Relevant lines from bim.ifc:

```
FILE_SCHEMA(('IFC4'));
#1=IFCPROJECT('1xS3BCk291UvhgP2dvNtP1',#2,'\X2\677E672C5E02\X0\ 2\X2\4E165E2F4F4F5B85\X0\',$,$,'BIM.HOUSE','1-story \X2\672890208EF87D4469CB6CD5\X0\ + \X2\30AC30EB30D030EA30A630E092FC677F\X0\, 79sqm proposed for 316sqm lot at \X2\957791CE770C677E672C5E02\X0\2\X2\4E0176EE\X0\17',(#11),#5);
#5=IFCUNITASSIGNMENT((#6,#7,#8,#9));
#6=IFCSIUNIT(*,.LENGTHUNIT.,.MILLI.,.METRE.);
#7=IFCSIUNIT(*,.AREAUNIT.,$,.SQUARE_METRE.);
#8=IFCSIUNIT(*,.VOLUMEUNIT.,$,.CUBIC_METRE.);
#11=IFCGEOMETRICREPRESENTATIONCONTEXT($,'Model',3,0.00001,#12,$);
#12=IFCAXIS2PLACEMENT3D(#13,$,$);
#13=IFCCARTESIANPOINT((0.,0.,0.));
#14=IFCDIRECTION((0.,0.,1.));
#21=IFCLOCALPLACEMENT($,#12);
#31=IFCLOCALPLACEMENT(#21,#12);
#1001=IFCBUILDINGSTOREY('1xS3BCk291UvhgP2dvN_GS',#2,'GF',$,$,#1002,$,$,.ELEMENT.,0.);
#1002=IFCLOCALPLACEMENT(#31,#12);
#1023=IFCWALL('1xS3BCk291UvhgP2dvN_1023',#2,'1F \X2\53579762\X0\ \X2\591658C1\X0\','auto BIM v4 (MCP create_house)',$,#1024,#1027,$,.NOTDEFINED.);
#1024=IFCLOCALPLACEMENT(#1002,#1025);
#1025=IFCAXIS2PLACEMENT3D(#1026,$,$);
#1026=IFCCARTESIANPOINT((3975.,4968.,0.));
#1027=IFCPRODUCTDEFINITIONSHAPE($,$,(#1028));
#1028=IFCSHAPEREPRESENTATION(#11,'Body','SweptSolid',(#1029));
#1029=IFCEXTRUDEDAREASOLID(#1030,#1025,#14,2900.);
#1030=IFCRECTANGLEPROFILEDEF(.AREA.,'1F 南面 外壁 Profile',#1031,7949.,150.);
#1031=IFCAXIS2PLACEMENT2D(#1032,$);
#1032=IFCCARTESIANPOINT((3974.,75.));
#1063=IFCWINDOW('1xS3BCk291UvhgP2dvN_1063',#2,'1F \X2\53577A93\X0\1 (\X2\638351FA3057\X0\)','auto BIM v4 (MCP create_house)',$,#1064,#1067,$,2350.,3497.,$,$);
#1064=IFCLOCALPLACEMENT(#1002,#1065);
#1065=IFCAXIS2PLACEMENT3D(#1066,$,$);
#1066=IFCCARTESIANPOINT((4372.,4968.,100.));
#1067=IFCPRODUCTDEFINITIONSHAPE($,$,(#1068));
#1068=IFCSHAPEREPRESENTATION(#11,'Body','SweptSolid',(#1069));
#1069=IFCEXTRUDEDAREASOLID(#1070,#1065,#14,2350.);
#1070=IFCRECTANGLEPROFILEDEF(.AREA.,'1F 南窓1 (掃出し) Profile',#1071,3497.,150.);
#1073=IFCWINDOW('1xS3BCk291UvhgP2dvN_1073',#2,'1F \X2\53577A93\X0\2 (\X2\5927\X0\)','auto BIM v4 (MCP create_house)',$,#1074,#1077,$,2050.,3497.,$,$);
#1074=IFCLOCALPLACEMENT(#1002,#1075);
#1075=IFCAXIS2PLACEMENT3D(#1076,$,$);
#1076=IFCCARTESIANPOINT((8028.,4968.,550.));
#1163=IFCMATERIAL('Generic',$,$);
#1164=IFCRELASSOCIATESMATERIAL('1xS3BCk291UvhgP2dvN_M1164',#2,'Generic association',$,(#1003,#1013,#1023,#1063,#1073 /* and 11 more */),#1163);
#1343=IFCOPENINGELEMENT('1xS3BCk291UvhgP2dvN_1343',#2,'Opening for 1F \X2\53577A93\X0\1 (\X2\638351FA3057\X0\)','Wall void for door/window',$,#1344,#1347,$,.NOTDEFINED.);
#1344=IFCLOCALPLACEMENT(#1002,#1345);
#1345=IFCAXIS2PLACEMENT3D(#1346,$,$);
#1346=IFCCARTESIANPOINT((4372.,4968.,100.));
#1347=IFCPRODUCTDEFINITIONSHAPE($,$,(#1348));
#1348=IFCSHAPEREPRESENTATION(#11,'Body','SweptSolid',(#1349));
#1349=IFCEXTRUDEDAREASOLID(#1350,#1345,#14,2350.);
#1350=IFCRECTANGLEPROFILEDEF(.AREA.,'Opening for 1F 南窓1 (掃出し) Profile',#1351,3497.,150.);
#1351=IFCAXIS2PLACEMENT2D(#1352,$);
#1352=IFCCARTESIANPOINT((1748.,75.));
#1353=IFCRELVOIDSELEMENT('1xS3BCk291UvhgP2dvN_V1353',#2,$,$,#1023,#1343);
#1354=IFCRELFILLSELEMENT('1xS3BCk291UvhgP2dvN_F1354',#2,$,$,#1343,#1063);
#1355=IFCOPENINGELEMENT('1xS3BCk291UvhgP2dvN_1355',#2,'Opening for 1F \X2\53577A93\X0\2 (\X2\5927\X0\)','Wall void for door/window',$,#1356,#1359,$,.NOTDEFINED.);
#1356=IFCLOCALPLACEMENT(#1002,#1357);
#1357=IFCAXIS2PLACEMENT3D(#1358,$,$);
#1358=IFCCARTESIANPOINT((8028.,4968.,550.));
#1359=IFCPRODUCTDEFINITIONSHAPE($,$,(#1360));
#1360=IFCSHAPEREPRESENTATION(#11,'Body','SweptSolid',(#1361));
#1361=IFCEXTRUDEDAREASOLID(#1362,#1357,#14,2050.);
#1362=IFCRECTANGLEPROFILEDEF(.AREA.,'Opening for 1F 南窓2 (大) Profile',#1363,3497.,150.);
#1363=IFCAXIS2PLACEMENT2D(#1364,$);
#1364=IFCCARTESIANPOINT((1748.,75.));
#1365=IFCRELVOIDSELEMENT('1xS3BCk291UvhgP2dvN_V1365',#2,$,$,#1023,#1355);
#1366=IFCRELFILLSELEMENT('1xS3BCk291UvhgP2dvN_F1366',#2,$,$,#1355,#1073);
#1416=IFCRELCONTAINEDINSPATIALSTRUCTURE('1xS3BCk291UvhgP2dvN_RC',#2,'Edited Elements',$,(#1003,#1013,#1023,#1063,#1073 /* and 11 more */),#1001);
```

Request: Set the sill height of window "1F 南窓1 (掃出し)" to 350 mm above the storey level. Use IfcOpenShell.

```python
import numpy as np
import ifcopenshell
import ifcopenshell.api.geometry
import ifcopenshell.geom
import ifcopenshell.util.element
import ifcopenshell.util.placement
import ifcopenshell.util.shape
import ifcopenshell.util.unit

model = ifcopenshell.open("bim.ifc")
unit_scale = ifcopenshell.util.unit.calculate_unit_scale(model)

window = model.by_guid("1xS3BCk291UvhgP2dvN_1063")
opening = window.FillsVoids[0].RelatingOpeningElement
storey = ifcopenshell.util.element.get_container(window, ifc_class="IfcBuildingStorey")
level = ifcopenshell.util.placement.get_local_placement(storey.ObjectPlacement)[2, 3]

# The opening's origin need not be at the sill, so measure its lowest point.
shape = ifcopenshell.geom.create_shape(ifcopenshell.geom.settings(), opening)
bottom = ifcopenshell.util.shape.get_shape_bottom_elevation(shape, shape.geometry) / unit_scale
dz = level + 0.35 / unit_scale - bottom

shift = np.array([0.0, 0.0, dz])
# The window is not placed relative to its opening, so move both.
for product in (opening, window):
    matrix = ifcopenshell.util.placement.get_local_placement(product.ObjectPlacement)
    matrix[:3, 3] += shift
    ifcopenshell.api.geometry.edit_object_placement(model, product=product, matrix=matrix, is_si=False)

print(f"moved by {dz * unit_scale:+.3f} m")

model.write("bim_updated.ifc")
```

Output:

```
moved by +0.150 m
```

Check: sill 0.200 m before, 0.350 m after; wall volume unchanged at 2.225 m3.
